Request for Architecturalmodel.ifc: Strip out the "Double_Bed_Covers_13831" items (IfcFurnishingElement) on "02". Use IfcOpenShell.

First a look at what the model holds.

```python
import ifcopenshell
import ifcopenshell.util.element

model = ifcopenshell.open("Architecturalmodel.ifc")
print(model.schema)
storey = next(s for s in model.by_type("IfcBuildingStorey") if s.Name == "02")
furniture = [e for e in ifcopenshell.util.element.get_decomposition(storey) if e.is_a("IfcFurnishingElement")]
seen = {}
for e in furniture:
    element_type = ifcopenshell.util.element.get_type(e)
    name = element_type.Name if element_type not in (None, e) else None
    seen[name] = seen.get(name, 0) + 1
for name, count in sorted(seen.items(), key=str):
    print(count, "x", name)
```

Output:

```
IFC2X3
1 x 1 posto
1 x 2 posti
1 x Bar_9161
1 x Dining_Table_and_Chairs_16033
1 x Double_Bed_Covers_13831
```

```python
import ifcopenshell
import ifcopenshell.api.root
import ifcopenshell.util.element

model = ifcopenshell.open("Architecturalmodel.ifc")

storey = next(s for s in model.by_type("IfcBuildingStorey") if s.Name == "02")
furniture = [e for e in ifcopenshell.util.element.get_decomposition(storey) if e.is_a("IfcFurnishingElement")]
targets = [e for e in furniture if (t := ifcopenshell.util.element.get_type(e)) not in (None, e) and t.Name == "Double_Bed_Covers_13831"]

for e in targets:
    ifcopenshell.api.root.remove_product(model, product=e)
print(len(targets), "removed")

model.write("Architecturalmodel-out.ifc")
```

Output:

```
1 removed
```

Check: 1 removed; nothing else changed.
